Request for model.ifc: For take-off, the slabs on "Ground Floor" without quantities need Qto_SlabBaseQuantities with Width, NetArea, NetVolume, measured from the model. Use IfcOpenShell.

First a look at what the model holds.

```python
import ifcopenshell
import ifcopenshell.util.element
import ifcopenshell.util.unit

model = ifcopenshell.open("model.ifc")
print(model.schema)
for unit_type in ("LENGTHUNIT", "AREAUNIT", "VOLUMEUNIT"):
    print(unit_type, ifcopenshell.util.unit.calculate_unit_scale(model, unit_type))
storey = next(s for s in model.by_type("IfcBuildingStorey") if s.Name == "Ground Floor")
slabs = [e for e in ifcopenshell.util.element.get_decomposition(storey) if e.is_a("IfcSlab")]
for e in sorted(slabs, key=lambda e: e.id()):
    print(e.id(), e.is_a(), e.Name, list(ifcopenshell.util.element.get_psets(e, qtos_only=True)), sep=" | ")
```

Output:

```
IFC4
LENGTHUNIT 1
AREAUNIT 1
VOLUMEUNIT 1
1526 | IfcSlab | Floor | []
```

```python
import ifcopenshell
import ifcopenshell.api.pset
import ifcopenshell.geom
import ifcopenshell.util.element
import ifcopenshell.util.shape
import ifcopenshell.util.unit

model = ifcopenshell.open("model.ifc")
unit_scale = ifcopenshell.util.unit.calculate_unit_scale(model)
area_scale = ifcopenshell.util.unit.calculate_unit_scale(model, "AREAUNIT")
volume_scale = ifcopenshell.util.unit.calculate_unit_scale(model, "VOLUMEUNIT")
settings = ifcopenshell.geom.settings()

storey = next(s for s in model.by_type("IfcBuildingStorey") if s.Name == "Ground Floor")
slabs = [e for e in ifcopenshell.util.element.get_decomposition(storey) if e.is_a("IfcSlab")]

for e in sorted(slabs, key=lambda e: e.id()):
    if ifcopenshell.util.element.get_psets(e, qtos_only=True, should_inherit=False):
        continue
    # Geometry comes back in metres, in the element's own axes.
    shape = ifcopenshell.geom.create_shape(settings, e)
    values = {
        "Width": ifcopenshell.util.shape.get_z(shape.geometry) / unit_scale,
        "NetArea": ifcopenshell.util.shape.get_footprint_area(shape.geometry) / area_scale,
        "NetVolume": ifcopenshell.util.shape.get_volume(shape.geometry) / volume_scale,
    }
    qto = ifcopenshell.api.pset.add_qto(model, product=e, name="Qto_SlabBaseQuantities")
    ifcopenshell.api.pset.edit_qto(model, qto=qto, properties=values)
    print(e.id(), {k: round(v, 3) for k, v in values.items()})

model.write("model_v2.ifc")
```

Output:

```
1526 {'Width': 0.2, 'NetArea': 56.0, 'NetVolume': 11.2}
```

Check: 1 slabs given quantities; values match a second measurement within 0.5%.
